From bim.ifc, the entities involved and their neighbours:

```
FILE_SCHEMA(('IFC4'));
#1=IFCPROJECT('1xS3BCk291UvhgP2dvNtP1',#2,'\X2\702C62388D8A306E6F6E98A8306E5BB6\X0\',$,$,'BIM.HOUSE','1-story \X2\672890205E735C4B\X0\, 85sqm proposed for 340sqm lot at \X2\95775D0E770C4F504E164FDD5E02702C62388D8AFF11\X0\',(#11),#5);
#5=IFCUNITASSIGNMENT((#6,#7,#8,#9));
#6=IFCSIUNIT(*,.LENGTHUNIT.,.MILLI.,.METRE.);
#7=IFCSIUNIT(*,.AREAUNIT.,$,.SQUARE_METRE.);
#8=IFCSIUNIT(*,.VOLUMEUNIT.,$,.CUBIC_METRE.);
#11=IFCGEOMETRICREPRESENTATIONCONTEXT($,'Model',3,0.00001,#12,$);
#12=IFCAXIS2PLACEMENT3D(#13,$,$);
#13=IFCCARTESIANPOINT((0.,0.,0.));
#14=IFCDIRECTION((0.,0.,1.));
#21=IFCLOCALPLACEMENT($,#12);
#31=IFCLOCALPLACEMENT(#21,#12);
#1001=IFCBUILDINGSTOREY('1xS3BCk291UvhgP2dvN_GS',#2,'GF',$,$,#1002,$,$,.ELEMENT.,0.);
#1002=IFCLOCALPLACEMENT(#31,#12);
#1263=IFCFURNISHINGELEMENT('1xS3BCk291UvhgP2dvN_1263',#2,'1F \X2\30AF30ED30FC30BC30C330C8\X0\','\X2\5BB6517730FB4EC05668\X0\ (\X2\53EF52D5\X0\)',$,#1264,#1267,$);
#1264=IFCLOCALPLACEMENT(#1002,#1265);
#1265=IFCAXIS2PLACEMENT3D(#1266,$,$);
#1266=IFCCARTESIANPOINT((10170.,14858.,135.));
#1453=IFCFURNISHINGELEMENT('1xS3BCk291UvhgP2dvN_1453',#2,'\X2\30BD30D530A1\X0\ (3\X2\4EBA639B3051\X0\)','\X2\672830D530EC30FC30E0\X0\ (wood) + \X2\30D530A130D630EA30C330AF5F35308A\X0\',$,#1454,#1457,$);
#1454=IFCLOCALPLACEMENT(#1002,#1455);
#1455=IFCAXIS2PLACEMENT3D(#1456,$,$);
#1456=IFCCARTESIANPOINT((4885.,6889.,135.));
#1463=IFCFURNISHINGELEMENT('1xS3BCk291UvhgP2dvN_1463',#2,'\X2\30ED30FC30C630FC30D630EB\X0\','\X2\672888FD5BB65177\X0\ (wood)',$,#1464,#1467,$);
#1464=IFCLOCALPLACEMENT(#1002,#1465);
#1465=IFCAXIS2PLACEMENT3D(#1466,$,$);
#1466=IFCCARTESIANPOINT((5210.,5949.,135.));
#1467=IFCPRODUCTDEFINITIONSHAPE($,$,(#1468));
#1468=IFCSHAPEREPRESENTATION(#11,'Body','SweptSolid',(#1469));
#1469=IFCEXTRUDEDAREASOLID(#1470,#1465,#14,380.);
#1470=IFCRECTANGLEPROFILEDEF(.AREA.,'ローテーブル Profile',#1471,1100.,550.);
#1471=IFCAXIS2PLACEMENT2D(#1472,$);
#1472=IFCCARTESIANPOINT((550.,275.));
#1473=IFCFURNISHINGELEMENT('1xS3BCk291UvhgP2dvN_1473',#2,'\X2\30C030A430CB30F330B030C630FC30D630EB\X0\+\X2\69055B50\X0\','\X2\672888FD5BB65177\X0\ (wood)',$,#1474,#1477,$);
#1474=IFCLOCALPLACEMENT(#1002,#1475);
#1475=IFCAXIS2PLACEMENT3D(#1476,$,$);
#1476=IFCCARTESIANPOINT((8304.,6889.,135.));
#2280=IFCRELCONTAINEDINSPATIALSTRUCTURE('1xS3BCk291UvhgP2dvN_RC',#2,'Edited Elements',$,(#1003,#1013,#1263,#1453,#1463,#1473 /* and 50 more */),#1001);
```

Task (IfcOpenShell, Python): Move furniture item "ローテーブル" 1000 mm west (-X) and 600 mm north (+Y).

```python
import ifcopenshell
import ifcopenshell.api.geometry
import ifcopenshell.util.placement
import ifcopenshell.util.unit

model = ifcopenshell.open("bim.ifc")
unit_scale = ifcopenshell.util.unit.calculate_unit_scale(model)

item = model.by_guid("1xS3BCk291UvhgP2dvN_1463")
matrix = ifcopenshell.util.placement.get_local_placement(item.ObjectPlacement)
matrix[0, 3] -= 1 / unit_scale
matrix[1, 3] += 0.6 / unit_scale
ifcopenshell.api.geometry.edit_object_placement(model, product=item, matrix=matrix, is_si=False)

print(ifcopenshell.util.placement.get_local_placement(item.ObjectPlacement).round(3) + 0.0)

model.write("bim_rev.ifc")
```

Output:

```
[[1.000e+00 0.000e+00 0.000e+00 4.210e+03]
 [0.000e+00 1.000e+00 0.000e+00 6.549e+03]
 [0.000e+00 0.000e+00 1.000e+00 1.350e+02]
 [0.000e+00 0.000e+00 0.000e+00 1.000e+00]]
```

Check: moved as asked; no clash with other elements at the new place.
